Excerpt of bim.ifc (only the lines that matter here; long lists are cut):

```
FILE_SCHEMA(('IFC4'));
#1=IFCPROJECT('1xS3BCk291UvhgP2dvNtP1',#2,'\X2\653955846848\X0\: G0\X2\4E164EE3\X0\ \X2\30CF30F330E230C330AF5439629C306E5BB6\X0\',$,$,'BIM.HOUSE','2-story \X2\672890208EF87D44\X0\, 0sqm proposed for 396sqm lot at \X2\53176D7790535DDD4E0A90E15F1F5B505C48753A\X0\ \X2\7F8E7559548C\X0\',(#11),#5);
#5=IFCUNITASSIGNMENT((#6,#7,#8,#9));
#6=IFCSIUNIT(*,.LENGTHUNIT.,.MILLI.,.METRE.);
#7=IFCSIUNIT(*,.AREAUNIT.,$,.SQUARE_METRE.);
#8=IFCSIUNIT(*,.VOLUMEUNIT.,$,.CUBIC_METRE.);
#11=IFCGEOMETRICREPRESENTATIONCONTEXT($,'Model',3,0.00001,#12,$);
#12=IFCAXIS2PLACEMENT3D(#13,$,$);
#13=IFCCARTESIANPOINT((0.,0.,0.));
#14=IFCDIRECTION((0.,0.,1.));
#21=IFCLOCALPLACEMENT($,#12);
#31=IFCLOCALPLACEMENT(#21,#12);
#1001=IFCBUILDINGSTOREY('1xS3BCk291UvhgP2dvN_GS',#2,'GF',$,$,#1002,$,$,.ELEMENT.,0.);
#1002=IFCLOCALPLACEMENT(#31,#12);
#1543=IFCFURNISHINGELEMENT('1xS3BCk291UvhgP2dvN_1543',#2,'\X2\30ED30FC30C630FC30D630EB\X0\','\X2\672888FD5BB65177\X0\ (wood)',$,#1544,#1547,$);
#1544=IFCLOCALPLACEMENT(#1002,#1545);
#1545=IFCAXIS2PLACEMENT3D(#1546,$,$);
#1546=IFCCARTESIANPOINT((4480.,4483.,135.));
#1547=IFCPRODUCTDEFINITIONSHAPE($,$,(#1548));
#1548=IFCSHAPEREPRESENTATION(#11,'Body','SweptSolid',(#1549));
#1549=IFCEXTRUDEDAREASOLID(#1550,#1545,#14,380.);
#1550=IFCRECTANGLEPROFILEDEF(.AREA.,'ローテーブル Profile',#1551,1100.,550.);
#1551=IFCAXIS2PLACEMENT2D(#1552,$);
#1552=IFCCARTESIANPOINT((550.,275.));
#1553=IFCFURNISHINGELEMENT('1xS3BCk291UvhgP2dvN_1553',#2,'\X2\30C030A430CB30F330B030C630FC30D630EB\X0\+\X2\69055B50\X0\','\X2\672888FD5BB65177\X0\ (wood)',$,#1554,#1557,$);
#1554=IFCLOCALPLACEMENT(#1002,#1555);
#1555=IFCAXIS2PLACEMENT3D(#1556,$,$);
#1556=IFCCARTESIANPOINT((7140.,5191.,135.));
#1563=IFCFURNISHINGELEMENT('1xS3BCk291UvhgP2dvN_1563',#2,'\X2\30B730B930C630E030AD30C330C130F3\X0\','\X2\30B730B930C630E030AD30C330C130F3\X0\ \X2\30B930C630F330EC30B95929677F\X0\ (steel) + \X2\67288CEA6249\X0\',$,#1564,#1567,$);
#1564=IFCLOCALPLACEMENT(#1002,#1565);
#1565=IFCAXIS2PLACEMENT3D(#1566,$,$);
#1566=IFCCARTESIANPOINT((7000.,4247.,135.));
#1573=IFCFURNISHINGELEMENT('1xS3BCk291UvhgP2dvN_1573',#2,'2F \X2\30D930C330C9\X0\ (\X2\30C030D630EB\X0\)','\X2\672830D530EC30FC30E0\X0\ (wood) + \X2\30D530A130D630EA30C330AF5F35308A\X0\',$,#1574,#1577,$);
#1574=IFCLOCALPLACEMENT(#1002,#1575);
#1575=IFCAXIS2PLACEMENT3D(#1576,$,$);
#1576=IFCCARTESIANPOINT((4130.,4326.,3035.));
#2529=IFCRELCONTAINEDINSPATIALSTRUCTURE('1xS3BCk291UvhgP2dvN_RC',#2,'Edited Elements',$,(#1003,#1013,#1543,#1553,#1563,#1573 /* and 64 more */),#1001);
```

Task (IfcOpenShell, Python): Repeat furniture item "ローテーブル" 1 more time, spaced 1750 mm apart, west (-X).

```python
import numpy as np
import ifcopenshell
import ifcopenshell.api.geometry
import ifcopenshell.api.root
import ifcopenshell.util.element
import ifcopenshell.util.placement
import ifcopenshell.util.unit

model = ifcopenshell.open("bim.ifc")
unit_scale = ifcopenshell.util.unit.calculate_unit_scale(model)


def reuse_history(source, copy):
    """copy_class also copies each property set's owner history, people and application; keep the originals."""
    for rel in copy.IsDefinedBy:
        if rel.is_a("IfcRelDefinesByProperties") and (history := rel.RelatingPropertyDefinition.OwnerHistory):
            rel.RelatingPropertyDefinition.OwnerHistory = source.OwnerHistory
            ifcopenshell.util.element.remove_deep2(model, history)


source = model.by_id(1543)
base = ifcopenshell.util.placement.get_local_placement(source.ObjectPlacement)
step = np.array([-1.0, 0.0, 0.0]) * 1.75 / unit_scale

for i in range(1, 2):
    copy = ifcopenshell.api.root.copy_class(model, product=source)
    copy.Representation = ifcopenshell.util.element.copy_deep(
        model, source.Representation, exclude=["IfcGeometricRepresentationContext", "IfcRepresentationMap"]
    )
    reuse_history(source, copy)
    matrix = base.copy()
    matrix[:3, 3] += i * step
    print("added at", matrix[:3, 3].round(3) + 0.0)
    ifcopenshell.api.geometry.edit_object_placement(model, product=copy, matrix=matrix, is_si=False)

model.write("bim_updated.ifc")
```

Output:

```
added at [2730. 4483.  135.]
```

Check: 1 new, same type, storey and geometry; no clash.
